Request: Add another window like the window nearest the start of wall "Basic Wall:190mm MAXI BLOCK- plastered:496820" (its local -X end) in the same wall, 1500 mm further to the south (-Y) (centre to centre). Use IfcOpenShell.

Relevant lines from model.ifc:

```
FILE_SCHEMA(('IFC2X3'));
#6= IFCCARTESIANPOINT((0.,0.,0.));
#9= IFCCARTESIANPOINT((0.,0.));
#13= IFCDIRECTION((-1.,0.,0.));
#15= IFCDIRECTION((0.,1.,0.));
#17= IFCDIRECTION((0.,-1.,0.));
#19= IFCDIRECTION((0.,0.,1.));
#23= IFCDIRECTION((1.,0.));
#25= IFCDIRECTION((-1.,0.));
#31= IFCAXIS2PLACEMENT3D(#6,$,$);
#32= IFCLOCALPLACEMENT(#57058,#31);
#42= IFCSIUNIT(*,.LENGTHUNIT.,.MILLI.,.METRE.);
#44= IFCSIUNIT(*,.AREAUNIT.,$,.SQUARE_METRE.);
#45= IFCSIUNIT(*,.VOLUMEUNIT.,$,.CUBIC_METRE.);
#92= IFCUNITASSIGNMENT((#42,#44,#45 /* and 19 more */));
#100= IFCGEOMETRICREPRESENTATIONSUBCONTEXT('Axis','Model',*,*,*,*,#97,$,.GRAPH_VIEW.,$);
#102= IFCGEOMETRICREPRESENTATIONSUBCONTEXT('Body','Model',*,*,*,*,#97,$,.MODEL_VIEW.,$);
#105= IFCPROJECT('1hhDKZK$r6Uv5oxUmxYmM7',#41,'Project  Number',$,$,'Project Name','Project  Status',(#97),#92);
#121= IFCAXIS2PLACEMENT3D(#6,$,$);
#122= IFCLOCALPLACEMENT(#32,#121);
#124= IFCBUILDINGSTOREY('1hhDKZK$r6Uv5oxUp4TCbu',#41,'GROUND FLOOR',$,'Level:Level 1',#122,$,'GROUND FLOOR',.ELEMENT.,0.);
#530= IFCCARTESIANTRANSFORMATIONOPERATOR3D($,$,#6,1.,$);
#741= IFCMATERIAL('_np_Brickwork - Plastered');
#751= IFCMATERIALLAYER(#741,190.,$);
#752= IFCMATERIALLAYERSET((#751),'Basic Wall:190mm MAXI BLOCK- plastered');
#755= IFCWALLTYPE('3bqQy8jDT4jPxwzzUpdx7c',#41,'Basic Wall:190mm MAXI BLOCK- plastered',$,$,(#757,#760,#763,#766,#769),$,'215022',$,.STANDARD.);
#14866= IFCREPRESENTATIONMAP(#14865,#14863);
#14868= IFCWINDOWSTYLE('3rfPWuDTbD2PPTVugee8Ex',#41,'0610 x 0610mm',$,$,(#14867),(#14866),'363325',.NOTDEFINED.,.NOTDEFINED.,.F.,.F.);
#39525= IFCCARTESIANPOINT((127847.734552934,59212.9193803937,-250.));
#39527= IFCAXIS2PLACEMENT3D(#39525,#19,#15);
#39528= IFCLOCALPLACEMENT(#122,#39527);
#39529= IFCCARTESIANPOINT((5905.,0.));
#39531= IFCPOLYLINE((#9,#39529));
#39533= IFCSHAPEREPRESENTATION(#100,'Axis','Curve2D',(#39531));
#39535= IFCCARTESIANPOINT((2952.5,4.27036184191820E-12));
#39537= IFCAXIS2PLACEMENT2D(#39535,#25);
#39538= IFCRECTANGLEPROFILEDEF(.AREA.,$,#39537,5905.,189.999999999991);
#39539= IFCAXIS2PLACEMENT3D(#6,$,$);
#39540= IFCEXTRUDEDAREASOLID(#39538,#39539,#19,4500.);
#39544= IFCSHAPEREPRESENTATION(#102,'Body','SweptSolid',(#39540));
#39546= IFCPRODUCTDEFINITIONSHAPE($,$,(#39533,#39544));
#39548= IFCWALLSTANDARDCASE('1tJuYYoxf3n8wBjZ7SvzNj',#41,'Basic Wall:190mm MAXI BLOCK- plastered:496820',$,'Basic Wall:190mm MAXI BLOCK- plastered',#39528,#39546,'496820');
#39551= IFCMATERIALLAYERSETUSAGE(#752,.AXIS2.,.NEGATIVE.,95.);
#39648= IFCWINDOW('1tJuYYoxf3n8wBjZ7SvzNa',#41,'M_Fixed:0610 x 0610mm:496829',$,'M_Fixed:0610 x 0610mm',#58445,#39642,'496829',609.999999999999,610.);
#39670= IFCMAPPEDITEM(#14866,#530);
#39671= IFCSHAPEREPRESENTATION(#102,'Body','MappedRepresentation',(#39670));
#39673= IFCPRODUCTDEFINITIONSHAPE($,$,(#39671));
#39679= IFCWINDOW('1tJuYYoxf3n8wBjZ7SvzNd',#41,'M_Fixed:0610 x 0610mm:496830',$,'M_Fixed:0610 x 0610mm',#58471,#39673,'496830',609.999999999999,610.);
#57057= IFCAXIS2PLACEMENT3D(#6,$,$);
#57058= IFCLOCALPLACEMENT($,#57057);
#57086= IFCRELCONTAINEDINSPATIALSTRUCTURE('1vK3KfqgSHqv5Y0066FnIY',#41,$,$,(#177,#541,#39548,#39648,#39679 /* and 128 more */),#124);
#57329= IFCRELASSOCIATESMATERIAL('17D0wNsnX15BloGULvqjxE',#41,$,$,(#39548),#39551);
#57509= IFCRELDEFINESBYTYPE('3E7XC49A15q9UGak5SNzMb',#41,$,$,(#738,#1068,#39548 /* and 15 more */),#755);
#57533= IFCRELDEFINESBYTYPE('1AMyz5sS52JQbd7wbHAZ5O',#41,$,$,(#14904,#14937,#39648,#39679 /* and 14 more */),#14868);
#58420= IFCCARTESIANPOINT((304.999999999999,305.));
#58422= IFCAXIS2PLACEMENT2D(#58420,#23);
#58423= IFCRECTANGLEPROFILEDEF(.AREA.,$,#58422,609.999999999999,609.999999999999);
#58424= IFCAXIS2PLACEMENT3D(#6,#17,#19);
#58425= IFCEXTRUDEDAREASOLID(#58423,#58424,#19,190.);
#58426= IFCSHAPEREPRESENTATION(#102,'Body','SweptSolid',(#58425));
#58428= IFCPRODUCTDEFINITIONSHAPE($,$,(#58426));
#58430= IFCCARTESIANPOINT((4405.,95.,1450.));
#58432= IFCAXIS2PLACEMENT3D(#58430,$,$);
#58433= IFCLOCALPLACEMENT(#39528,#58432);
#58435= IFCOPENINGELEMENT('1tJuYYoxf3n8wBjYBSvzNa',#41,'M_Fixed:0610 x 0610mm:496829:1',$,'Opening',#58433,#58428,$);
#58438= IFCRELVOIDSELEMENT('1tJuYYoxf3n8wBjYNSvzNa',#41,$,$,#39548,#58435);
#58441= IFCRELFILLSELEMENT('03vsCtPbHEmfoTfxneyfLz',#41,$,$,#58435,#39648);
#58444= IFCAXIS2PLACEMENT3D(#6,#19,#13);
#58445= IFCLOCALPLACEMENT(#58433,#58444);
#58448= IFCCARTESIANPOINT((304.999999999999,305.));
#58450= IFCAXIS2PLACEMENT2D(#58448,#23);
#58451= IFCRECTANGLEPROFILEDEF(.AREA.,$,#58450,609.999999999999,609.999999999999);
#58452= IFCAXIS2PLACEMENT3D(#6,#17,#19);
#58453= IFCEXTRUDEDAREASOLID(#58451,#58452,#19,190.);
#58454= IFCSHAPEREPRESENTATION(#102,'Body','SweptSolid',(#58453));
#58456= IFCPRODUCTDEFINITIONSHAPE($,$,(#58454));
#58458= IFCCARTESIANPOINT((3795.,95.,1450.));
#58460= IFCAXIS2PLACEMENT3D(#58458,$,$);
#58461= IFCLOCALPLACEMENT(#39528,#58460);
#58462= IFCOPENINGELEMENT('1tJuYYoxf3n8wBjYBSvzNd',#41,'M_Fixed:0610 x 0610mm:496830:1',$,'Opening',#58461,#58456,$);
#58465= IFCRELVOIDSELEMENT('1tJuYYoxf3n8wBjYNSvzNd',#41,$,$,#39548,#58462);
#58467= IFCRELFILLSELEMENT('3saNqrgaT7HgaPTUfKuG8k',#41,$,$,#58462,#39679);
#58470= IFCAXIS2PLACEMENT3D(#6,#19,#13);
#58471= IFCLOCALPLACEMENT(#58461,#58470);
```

```python
import ifcopenshell
import ifcopenshell.api.feature
import ifcopenshell.api.geometry
import ifcopenshell.api.root
import ifcopenshell.geom
import ifcopenshell.util.element
import ifcopenshell.util.placement
import ifcopenshell.util.shape
import ifcopenshell.util.unit

model = ifcopenshell.open("model.ifc")
unit_scale = ifcopenshell.util.unit.calculate_unit_scale(model)
settings = ifcopenshell.geom.settings()


def volume(element):
    """Net volume in cubic metres, openings subtracted."""
    shape = ifcopenshell.geom.create_shape(settings, element)
    return ifcopenshell.util.shape.get_volume(shape.geometry)


def reuse_history(source, copy):
    """copy_class also copies each property set's owner history, people and application; keep the originals."""
    for rel in copy.IsDefinedBy:
        if rel.is_a("IfcRelDefinesByProperties") and (history := rel.RelatingPropertyDefinition.OwnerHistory):
            rel.RelatingPropertyDefinition.OwnerHistory = source.OwnerHistory
            ifcopenshell.util.element.remove_deep2(model, history)


window = model.by_guid("1tJuYYoxf3n8wBjZ7SvzNd")
opening = window.FillsVoids[0].RelatingOpeningElement
wall = opening.VoidsElements[0].RelatingBuildingElement
before = volume(wall)
shift = ifcopenshell.util.placement.get_local_placement(wall.ObjectPlacement)[:3, 0] * -1.5 / unit_scale

# copy_class copies the void relationship, type, container and properties, but no geometry.
new_opening = ifcopenshell.api.root.copy_class(model, product=opening)
new_opening.Representation = ifcopenshell.util.element.copy_deep(
    model, opening.Representation, exclude=["IfcGeometricRepresentationContext", "IfcRepresentationMap"]
)
new_opening.Name = "M_Fixed:0610 x 0610mm"
new_window = ifcopenshell.api.root.copy_class(model, product=window)
new_window.Representation = ifcopenshell.util.element.copy_deep(
    model, window.Representation, exclude=["IfcGeometricRepresentationContext", "IfcRepresentationMap"]
)
new_window.Name = "M_Fixed:0610 x 0610mm"
new_window.Tag = None
reuse_history(window, new_window)
fills = ifcopenshell.api.feature.add_filling(model, opening=new_opening, element=new_window)
fills.OwnerHistory = new_window.OwnerHistory  # required in IFC2X3

for old, new in ((opening, new_opening), (window, new_window)):
    matrix = ifcopenshell.util.placement.get_local_placement(old.ObjectPlacement)
    matrix[:3, 3] += shift
    ifcopenshell.api.geometry.edit_object_placement(model, product=new, matrix=matrix, is_si=False)

after = volume(wall)

print(f"wall volume {before:.3f} -> {after:.3f} m3")

model.write("model_v2.ifc")
```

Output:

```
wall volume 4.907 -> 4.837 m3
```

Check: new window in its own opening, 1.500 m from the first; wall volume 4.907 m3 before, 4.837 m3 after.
